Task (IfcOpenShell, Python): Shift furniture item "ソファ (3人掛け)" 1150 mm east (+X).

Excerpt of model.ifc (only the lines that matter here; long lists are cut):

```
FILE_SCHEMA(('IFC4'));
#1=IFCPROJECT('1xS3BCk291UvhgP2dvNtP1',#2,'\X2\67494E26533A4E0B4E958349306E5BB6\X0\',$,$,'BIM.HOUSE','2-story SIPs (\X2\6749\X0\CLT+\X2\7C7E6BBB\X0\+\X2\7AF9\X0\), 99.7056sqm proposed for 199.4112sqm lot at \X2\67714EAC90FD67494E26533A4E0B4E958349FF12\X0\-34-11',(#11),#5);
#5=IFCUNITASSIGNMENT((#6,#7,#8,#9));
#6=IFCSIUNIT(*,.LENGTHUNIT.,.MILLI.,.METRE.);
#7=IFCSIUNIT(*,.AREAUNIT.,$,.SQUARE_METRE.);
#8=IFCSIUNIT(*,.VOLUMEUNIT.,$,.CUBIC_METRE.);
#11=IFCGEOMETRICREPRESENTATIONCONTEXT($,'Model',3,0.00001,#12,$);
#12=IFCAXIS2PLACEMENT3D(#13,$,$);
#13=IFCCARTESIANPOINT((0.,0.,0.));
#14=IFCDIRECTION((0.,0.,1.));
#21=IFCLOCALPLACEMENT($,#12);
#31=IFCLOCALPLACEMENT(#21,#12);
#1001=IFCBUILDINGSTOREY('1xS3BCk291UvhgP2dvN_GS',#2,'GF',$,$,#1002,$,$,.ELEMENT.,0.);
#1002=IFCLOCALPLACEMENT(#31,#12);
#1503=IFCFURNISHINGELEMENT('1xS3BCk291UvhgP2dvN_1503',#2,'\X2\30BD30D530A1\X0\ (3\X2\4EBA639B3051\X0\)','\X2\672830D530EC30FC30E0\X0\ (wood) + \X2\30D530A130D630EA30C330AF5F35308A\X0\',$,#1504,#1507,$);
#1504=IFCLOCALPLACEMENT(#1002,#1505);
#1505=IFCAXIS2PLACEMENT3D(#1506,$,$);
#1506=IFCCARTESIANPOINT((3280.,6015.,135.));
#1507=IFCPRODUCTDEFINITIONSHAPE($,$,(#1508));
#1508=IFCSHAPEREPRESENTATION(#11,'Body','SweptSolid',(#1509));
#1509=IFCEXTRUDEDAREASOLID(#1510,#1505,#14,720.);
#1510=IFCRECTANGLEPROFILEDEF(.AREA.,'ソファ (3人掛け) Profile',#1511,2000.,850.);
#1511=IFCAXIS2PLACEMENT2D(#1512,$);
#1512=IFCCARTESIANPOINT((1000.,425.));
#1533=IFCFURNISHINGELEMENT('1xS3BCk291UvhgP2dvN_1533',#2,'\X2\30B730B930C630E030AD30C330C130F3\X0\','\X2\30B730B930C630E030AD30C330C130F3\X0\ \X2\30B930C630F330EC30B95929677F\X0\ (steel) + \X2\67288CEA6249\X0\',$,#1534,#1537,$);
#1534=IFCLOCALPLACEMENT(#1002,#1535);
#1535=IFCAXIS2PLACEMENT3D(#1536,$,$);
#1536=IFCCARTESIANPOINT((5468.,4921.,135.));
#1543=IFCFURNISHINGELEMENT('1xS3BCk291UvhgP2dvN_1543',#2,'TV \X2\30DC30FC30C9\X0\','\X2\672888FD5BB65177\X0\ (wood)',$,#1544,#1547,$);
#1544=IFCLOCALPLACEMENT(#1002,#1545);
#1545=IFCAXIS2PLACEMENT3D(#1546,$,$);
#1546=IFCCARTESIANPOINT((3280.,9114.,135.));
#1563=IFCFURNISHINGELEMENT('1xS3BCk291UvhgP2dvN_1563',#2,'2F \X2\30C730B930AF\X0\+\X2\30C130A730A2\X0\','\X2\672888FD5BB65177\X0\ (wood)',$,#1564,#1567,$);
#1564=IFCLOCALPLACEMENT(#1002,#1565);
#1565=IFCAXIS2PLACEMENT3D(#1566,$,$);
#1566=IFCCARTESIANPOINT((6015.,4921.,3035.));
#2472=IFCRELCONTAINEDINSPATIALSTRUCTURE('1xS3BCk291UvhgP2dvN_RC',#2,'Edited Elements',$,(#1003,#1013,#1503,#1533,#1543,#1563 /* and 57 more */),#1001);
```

```python
import ifcopenshell
import ifcopenshell.api.geometry
import ifcopenshell.util.placement
import ifcopenshell.util.unit

model = ifcopenshell.open("model.ifc")
unit_scale = ifcopenshell.util.unit.calculate_unit_scale(model)

item = model.by_guid("1xS3BCk291UvhgP2dvN_1503")
matrix = ifcopenshell.util.placement.get_local_placement(item.ObjectPlacement)
matrix[0, 3] += 1.15 / unit_scale
ifcopenshell.api.geometry.edit_object_placement(model, product=item, matrix=matrix, is_si=False)

print(ifcopenshell.util.placement.get_local_placement(item.ObjectPlacement).round(3) + 0.0)

model.write("model_v2.ifc")
```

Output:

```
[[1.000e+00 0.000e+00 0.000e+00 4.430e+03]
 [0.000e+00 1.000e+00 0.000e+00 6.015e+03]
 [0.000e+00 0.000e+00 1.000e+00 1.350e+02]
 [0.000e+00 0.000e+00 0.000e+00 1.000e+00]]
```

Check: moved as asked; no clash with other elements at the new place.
